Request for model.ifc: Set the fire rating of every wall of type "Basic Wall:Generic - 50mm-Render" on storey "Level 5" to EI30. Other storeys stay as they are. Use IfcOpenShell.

First a look at what the model holds.

```python
import ifcopenshell
import ifcopenshell.util.element

model = ifcopenshell.open("model.ifc")
print(model.schema)
storey = next(s for s in model.by_type("IfcBuildingStorey") if s.Name == "Level 5")
walls = [e for e in ifcopenshell.util.element.get_decomposition(storey) if e.is_a("IfcWall")]
seen = {}
for e in walls:
    element_type = ifcopenshell.util.element.get_type(e)
    key = (element_type.Name if element_type != e and element_type else None, ifcopenshell.util.element.get_pset(e, "Pset_WallCommon", "FireRating"))
    seen[key] = seen.get(key, 0) + 1
for (name, value), count in sorted(seen.items(), key=str):
    print(count, "x", name, "|", value)
```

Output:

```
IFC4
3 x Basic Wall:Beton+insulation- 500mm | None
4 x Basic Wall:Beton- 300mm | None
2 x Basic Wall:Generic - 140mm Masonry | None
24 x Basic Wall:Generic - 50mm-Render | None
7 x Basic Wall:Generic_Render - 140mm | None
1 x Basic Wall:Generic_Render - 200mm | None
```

```python
import ifcopenshell
import ifcopenshell.api.pset
import ifcopenshell.util.element

model = ifcopenshell.open("model.ifc")

storey = next(s for s in model.by_type("IfcBuildingStorey") if s.Name == "Level 5")
walls = [e for e in ifcopenshell.util.element.get_decomposition(storey) if e.is_a("IfcWall")]

count = 0
for e in walls:
    element_type = ifcopenshell.util.element.get_type(e)
    if element_type in (None, e) or element_type.Name != "Basic Wall:Generic - 50mm-Render":
        continue
    # add_pset returns the element's existing set when there is one.
    pset = ifcopenshell.api.pset.add_pset(model, product=e, name="Pset_WallCommon")
    ifcopenshell.api.pset.edit_pset(model, pset=pset, properties={"FireRating": "EI30"})
    count += 1

print(count, "walls updated")

model.write("model_edited.ifc")
```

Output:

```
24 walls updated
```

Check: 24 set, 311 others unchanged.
